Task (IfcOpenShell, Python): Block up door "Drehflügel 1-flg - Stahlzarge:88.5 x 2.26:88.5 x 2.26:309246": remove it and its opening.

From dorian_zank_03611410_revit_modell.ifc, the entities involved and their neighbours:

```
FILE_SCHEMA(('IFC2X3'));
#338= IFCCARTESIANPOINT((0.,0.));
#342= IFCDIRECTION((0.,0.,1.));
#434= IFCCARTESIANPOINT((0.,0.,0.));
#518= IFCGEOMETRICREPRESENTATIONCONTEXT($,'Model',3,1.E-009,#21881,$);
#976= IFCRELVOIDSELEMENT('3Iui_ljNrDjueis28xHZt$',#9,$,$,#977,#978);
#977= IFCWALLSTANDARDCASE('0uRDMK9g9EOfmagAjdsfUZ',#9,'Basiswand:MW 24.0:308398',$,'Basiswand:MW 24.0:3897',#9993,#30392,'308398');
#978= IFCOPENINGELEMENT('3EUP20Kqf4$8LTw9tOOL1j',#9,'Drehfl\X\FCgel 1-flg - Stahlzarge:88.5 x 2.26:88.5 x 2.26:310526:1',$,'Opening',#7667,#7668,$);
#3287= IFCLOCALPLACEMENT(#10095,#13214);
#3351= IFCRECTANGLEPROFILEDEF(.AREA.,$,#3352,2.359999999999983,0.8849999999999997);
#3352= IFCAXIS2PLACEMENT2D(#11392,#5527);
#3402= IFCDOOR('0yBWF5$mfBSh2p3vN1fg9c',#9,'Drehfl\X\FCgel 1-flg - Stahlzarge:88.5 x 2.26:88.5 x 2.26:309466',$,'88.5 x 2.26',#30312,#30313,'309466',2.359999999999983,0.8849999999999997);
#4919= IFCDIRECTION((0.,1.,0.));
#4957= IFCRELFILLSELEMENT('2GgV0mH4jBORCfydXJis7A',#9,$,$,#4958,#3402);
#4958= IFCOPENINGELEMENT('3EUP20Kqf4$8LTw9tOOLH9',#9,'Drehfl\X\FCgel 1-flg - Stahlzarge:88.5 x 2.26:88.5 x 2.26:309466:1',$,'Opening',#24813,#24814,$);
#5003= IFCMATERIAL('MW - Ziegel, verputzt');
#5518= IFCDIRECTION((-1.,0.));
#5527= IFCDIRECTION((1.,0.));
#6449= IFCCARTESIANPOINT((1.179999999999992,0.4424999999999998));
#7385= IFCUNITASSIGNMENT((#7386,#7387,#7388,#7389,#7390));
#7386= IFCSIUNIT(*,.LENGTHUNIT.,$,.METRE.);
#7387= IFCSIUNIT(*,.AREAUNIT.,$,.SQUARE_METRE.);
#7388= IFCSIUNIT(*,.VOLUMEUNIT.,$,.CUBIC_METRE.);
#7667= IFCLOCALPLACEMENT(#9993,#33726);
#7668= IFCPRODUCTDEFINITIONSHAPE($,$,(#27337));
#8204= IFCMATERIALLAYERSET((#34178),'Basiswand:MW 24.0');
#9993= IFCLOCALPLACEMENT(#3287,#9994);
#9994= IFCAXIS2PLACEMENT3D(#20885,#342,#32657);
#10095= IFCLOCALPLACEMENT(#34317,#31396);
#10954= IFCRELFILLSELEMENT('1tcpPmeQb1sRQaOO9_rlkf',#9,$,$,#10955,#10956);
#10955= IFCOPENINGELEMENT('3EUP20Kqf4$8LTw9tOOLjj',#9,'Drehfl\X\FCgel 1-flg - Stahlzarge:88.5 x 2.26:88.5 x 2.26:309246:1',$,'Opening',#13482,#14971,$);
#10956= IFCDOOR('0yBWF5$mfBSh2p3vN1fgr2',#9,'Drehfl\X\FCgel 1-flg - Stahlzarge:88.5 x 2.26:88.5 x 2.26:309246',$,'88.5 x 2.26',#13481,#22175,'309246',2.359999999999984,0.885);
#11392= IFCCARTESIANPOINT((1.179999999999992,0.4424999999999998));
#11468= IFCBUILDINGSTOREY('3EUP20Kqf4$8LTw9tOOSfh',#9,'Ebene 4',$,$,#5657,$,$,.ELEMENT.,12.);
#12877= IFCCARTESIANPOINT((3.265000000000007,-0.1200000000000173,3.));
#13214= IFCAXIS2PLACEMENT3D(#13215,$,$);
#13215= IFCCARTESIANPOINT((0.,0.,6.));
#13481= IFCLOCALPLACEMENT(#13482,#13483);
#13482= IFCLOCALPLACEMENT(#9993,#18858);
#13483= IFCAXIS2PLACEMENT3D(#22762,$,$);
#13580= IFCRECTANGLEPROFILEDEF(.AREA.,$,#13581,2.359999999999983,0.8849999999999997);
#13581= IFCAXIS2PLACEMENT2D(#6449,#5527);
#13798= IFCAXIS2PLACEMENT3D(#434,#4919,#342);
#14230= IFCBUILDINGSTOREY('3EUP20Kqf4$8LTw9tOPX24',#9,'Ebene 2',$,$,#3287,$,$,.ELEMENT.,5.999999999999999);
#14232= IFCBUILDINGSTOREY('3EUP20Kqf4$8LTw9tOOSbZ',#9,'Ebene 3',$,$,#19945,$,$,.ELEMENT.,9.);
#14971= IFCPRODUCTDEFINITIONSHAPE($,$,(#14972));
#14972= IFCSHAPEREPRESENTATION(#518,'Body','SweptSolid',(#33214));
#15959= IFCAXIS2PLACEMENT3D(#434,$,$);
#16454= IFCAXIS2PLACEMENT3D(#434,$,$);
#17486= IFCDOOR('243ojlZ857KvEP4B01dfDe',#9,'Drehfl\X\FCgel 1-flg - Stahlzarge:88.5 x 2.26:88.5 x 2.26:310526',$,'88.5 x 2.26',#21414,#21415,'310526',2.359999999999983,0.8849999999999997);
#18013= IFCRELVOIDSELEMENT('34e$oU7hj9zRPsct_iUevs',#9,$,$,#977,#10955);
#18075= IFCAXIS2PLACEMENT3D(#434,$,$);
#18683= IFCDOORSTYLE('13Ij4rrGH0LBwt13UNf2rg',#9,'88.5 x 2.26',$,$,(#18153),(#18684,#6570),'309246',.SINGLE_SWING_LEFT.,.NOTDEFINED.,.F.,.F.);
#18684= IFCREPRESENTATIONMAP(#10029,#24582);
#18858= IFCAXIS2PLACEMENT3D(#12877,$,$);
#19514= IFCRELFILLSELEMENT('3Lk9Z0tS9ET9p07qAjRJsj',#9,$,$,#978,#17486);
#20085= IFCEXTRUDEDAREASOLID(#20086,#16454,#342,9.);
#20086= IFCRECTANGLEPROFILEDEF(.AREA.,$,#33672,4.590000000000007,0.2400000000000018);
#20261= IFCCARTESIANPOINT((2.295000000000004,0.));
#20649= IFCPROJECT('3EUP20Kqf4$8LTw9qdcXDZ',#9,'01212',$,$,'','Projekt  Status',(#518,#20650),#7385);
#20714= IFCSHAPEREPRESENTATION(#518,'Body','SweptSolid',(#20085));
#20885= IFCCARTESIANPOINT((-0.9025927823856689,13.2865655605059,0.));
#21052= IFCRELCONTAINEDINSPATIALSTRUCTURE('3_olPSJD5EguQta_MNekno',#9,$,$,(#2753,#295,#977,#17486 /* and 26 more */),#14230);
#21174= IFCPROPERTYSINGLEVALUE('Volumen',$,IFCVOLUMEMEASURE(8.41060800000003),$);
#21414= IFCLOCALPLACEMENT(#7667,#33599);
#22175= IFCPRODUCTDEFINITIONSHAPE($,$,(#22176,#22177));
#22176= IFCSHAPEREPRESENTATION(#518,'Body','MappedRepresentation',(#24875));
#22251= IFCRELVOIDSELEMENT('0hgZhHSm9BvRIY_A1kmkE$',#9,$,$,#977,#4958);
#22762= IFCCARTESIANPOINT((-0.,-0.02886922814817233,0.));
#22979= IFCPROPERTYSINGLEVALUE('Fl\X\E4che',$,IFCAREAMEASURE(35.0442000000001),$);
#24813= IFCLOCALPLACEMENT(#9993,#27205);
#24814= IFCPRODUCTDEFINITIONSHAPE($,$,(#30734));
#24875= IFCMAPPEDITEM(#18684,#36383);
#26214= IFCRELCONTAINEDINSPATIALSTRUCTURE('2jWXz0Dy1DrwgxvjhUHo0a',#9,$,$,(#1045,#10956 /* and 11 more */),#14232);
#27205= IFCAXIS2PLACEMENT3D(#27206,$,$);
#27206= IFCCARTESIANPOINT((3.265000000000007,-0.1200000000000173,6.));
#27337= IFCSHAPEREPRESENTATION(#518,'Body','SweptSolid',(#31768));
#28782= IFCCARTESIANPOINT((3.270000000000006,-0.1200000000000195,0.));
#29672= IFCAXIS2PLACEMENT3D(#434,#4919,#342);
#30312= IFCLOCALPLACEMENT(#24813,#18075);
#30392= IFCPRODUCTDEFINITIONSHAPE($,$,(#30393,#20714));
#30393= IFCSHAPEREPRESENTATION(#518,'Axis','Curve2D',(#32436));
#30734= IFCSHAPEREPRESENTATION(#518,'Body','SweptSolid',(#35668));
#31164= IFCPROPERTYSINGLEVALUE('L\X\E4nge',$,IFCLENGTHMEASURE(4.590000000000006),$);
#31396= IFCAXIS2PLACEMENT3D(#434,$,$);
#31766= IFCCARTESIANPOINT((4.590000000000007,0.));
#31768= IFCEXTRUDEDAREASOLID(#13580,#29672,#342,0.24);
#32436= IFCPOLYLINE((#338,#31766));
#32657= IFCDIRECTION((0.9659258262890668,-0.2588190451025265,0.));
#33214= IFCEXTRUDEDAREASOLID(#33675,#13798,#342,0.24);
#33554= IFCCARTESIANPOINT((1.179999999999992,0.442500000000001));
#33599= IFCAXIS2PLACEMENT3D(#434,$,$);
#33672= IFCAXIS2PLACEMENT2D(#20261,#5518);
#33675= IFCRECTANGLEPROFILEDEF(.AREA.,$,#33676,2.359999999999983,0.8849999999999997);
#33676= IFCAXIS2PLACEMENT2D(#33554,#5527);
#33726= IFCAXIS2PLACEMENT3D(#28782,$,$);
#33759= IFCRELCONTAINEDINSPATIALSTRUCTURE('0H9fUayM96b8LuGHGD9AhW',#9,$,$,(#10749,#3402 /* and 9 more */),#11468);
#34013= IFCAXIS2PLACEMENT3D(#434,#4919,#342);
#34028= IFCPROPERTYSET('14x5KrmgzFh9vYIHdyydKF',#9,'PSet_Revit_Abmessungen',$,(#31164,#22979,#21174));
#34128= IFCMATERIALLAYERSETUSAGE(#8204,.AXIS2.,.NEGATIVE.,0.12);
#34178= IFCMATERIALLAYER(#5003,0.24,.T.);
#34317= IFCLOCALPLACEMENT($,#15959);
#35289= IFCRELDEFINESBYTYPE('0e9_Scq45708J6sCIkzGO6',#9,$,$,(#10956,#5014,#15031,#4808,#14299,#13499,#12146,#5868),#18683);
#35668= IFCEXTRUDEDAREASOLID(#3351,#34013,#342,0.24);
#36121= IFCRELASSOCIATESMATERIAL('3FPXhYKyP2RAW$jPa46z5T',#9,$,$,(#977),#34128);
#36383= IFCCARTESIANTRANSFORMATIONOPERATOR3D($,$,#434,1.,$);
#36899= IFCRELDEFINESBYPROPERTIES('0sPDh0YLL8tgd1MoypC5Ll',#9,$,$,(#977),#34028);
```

```python
import ifcopenshell
import ifcopenshell.api.feature
import ifcopenshell.api.pset
import ifcopenshell.api.root
import ifcopenshell.geom
import ifcopenshell.util.element
import ifcopenshell.util.shape
import ifcopenshell.util.unit

model = ifcopenshell.open("dorian_zank_03611410_revit_modell.ifc")
area_scale = ifcopenshell.util.unit.calculate_unit_scale(model, "AREAUNIT")
volume_scale = ifcopenshell.util.unit.calculate_unit_scale(model, "VOLUMEUNIT")
settings = ifcopenshell.geom.settings()


def volume(element):
    """Net volume in cubic metres, openings subtracted."""
    shape = ifcopenshell.geom.create_shape(settings, element)
    return ifcopenshell.util.shape.get_volume(shape.geometry)


door = model.by_id(10956)
opening = door.FillsVoids[0].RelatingOpeningElement
wall = opening.VoidsElements[0].RelatingBuildingElement
before = volume(wall)

ifcopenshell.api.root.remove_product(model, product=door)
ifcopenshell.api.feature.remove_feature(model, feature=opening)

after = volume(wall)
thickness = 0.24  # wall thickness in metres

# Update the wall's stored quantities.
pset = model.by_id(ifcopenshell.util.element.get_pset(wall, "PSet_Revit_Abmessungen", should_inherit=False)["id"])
ifcopenshell.api.pset.edit_pset(model, pset=pset, properties={
    "Fläche": model.create_entity("IfcAreaMeasure", after / thickness / area_scale),
    "Volumen": model.create_entity("IfcVolumeMeasure", after / volume_scale),
})

print(f"wall volume {before:.3f} -> {after:.3f} m3")

model.write("dorian_zank_03611410_revit_modell_updated.ifc")
```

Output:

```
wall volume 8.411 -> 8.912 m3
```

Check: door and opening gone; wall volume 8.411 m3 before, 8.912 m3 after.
